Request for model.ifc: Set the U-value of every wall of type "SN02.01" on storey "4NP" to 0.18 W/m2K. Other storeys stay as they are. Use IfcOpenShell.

First a look at what the model holds.

```python
import ifcopenshell
import ifcopenshell.util.element

model = ifcopenshell.open("model.ifc")
print(model.schema)
storey = next(s for s in model.by_type("IfcBuildingStorey") if s.Name == "4NP")
walls = [e for e in ifcopenshell.util.element.get_decomposition(storey) if e.is_a("IfcWall")]
seen = {}
for e in walls:
    element_type = ifcopenshell.util.element.get_type(e)
    key = (element_type.Name if element_type != e and element_type else None, ifcopenshell.util.element.get_pset(e, "Pset_WallCommon", "ThermalTransmittance"))
    seen[key] = seen.get(key, 0) + 1
for (name, value), count in sorted(seen.items(), key=str):
    print(count, "x", name, "|", value)
```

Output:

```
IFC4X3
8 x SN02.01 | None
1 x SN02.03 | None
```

```python
import ifcopenshell
import ifcopenshell.api.pset
import ifcopenshell.util.element

model = ifcopenshell.open("model.ifc")

storey = next(s for s in model.by_type("IfcBuildingStorey") if s.Name == "4NP")
walls = [e for e in ifcopenshell.util.element.get_decomposition(storey) if e.is_a("IfcWall")]

count = 0
for e in walls:
    element_type = ifcopenshell.util.element.get_type(e)
    if element_type in (None, e) or element_type.Name != "SN02.01":
        continue
    # add_pset returns the element's existing set when there is one.
    pset = ifcopenshell.api.pset.add_pset(model, product=e, name="Pset_WallCommon")
    ifcopenshell.api.pset.edit_pset(model, pset=pset, properties={"ThermalTransmittance": 0.18})
    count += 1

print(count, "walls updated")

model.write("model_edited.ifc")
```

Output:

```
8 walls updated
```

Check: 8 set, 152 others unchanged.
